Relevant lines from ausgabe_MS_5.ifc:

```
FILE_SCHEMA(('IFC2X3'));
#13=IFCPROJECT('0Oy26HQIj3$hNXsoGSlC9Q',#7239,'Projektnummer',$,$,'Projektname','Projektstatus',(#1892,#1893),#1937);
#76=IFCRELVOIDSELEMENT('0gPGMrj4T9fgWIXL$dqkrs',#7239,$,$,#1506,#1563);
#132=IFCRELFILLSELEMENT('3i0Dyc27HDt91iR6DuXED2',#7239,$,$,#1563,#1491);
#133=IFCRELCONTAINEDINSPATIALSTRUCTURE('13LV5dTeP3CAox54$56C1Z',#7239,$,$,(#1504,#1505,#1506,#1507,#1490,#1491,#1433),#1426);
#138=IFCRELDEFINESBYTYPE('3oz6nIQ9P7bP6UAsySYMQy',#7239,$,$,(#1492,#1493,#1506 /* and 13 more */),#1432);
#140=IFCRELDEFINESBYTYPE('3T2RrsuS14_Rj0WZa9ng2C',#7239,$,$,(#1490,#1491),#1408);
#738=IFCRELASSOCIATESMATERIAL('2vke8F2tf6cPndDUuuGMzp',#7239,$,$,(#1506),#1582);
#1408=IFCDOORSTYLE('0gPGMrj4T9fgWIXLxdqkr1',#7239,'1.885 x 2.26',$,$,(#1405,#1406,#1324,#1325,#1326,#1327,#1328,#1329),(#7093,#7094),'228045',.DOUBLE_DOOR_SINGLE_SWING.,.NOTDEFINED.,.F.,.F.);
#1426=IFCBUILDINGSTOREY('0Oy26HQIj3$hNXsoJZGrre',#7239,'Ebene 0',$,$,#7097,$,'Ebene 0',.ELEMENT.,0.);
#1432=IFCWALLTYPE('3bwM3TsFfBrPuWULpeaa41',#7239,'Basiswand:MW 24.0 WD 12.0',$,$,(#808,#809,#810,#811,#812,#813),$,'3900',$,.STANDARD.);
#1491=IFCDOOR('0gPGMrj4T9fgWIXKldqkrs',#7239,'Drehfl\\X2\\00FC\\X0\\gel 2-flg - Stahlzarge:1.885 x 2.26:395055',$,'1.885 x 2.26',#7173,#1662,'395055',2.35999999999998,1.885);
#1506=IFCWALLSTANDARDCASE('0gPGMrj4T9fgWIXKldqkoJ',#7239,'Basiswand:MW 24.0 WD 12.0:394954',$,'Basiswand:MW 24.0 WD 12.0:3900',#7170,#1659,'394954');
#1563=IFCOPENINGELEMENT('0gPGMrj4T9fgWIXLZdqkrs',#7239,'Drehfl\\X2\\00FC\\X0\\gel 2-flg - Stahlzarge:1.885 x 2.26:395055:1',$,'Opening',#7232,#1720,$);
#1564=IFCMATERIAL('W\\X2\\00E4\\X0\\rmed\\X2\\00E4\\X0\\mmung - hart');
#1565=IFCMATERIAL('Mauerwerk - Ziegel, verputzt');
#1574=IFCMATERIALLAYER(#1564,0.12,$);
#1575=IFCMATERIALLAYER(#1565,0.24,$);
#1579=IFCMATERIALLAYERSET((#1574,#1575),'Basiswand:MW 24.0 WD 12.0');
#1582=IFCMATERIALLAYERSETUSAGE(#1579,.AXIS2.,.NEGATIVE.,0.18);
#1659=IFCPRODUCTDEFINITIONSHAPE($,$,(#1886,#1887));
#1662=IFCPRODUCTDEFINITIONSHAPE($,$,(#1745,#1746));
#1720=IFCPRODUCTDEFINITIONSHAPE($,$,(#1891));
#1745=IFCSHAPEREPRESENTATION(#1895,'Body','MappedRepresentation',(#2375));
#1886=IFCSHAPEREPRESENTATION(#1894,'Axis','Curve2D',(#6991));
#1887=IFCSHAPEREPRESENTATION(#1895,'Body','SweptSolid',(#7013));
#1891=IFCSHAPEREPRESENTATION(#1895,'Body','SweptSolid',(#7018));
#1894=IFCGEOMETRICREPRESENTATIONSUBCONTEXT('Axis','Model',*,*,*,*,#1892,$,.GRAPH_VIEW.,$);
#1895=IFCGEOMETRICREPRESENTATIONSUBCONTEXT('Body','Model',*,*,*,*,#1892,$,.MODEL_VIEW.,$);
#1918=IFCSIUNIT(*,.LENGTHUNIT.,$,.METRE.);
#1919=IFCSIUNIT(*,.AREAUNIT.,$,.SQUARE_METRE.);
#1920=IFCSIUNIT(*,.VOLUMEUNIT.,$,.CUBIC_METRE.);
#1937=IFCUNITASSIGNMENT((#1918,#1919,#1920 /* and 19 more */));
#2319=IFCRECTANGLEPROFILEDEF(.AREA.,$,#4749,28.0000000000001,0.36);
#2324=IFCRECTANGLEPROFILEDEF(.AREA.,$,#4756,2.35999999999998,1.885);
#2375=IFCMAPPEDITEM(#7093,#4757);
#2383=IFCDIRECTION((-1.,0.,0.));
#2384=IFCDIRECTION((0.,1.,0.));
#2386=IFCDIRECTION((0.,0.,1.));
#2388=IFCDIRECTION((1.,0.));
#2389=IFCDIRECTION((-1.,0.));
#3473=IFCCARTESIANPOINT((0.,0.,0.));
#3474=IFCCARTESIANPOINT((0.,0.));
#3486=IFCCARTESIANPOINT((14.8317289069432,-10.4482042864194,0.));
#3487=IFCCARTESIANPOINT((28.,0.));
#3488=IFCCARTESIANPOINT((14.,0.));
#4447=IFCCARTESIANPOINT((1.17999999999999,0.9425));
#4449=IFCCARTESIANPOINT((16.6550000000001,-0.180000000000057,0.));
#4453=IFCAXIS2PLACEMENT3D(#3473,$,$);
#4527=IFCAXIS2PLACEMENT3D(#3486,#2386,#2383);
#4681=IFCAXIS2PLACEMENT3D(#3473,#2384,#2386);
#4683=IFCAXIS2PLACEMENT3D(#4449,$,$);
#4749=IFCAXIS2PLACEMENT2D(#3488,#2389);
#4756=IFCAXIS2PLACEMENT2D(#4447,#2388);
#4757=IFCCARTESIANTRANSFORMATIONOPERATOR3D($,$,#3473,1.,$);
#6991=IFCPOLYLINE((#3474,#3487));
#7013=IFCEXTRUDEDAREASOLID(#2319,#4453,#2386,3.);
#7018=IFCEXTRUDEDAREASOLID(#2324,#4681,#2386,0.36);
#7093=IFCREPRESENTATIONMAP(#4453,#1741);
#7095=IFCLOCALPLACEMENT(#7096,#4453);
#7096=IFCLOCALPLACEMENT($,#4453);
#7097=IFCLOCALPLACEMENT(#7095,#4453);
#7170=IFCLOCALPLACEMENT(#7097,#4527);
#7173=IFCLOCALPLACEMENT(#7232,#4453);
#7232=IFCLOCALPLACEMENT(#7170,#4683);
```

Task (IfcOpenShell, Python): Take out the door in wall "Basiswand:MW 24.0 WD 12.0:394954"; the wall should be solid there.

```python
import ifcopenshell
import ifcopenshell.api.feature
import ifcopenshell.api.root
import ifcopenshell.geom
import ifcopenshell.util.shape

model = ifcopenshell.open("ausgabe_MS_5.ifc")
settings = ifcopenshell.geom.settings()


def volume(element):
    """Net volume in cubic metres, openings subtracted."""
    shape = ifcopenshell.geom.create_shape(settings, element)
    return ifcopenshell.util.shape.get_volume(shape.geometry)


door = model.by_guid("0gPGMrj4T9fgWIXKldqkrs")
opening = door.FillsVoids[0].RelatingOpeningElement
wall = opening.VoidsElements[0].RelatingBuildingElement
before = volume(wall)

ifcopenshell.api.root.remove_product(model, product=door)
ifcopenshell.api.feature.remove_feature(model, feature=opening)

after = volume(wall)

print(f"wall volume {before:.3f} -> {after:.3f} m3")

model.write("ausgabe_MS_5_v2.ifc")
```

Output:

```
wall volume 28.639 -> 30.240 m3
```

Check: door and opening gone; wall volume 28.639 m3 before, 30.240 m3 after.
